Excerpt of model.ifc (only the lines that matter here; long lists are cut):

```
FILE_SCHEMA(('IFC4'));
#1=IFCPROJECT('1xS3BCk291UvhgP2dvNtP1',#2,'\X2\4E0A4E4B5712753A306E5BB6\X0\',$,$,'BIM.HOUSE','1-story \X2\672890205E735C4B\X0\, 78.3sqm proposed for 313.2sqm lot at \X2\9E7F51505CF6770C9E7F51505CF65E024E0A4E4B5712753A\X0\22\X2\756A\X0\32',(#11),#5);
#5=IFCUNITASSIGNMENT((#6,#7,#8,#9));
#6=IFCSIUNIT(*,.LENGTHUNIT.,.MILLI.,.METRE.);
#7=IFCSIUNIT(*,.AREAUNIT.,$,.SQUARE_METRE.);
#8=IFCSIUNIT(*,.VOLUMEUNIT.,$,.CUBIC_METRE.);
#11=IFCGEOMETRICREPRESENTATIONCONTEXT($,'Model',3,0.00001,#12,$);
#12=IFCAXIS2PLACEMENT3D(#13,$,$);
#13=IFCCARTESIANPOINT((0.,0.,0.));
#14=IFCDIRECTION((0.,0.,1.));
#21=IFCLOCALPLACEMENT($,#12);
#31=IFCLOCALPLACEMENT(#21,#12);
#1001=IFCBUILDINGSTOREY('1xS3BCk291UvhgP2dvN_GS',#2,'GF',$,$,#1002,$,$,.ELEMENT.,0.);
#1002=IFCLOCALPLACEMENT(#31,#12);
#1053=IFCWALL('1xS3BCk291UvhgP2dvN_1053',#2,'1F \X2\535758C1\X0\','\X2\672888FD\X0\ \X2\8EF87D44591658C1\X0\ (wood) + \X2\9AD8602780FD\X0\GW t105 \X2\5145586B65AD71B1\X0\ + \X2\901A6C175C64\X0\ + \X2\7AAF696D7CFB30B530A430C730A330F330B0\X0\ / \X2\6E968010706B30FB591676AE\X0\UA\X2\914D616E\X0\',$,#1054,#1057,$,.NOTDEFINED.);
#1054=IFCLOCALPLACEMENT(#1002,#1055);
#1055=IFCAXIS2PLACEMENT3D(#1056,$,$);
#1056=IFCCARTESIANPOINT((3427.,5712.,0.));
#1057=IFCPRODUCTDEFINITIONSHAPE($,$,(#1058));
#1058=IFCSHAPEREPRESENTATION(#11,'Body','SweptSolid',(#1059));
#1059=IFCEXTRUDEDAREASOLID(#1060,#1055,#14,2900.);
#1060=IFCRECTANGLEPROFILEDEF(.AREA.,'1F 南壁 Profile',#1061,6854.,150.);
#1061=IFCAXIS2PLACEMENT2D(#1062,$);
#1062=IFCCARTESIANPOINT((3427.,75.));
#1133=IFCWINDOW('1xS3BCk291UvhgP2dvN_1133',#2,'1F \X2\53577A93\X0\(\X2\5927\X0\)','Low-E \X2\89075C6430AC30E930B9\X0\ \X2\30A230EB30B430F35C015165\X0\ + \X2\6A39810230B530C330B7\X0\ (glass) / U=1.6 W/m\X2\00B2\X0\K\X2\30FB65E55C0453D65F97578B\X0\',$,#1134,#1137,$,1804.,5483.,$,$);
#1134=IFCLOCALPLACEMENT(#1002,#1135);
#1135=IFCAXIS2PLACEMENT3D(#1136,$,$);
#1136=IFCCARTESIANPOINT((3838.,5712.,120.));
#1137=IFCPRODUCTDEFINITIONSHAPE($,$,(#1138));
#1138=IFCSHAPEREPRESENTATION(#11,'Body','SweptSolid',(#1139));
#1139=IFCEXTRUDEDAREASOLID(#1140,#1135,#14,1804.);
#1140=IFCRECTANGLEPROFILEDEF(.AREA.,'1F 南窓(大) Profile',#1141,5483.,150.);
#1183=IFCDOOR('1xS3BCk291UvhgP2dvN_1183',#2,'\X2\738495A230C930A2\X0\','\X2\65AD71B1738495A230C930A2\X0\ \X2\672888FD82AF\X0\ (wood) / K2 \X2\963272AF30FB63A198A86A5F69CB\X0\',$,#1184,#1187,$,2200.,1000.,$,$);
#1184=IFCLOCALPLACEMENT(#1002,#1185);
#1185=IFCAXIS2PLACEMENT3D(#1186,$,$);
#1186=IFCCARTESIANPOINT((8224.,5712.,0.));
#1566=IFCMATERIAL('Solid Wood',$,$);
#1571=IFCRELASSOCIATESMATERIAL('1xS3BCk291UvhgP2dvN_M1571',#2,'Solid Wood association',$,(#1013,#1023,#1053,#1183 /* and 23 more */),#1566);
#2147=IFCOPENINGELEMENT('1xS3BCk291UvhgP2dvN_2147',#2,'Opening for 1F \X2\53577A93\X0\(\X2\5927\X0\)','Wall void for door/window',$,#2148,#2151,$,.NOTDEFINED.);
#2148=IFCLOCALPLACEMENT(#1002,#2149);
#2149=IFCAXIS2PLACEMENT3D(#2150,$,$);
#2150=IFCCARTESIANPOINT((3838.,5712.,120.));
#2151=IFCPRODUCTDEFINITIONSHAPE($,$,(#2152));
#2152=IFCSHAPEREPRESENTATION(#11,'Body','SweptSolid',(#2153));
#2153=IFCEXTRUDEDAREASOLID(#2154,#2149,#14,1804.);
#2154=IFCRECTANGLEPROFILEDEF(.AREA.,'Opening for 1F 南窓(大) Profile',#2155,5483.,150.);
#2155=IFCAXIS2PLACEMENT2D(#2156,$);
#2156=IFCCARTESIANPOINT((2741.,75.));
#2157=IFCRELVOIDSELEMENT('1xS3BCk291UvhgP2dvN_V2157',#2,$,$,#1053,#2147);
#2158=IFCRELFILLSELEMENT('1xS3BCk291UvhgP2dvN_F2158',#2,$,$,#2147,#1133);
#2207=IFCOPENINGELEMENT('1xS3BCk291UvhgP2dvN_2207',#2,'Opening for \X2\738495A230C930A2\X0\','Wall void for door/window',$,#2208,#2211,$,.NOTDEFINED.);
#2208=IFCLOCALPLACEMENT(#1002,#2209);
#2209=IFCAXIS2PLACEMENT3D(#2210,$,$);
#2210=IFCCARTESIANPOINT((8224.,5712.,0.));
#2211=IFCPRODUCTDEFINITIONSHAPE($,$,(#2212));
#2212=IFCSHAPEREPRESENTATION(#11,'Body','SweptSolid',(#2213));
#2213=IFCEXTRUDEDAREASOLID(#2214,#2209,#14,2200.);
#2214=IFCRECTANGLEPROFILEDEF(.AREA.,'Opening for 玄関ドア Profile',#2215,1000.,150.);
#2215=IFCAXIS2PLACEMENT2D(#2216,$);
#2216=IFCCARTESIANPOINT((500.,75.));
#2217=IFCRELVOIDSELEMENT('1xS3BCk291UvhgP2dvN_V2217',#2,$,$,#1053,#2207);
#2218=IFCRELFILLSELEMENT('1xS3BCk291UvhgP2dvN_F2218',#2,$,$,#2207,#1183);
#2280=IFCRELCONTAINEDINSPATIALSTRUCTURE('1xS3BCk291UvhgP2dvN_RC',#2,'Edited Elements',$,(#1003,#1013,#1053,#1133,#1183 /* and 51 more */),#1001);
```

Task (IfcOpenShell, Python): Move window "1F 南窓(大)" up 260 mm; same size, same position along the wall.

```python
import numpy as np
import ifcopenshell
import ifcopenshell.api.geometry
import ifcopenshell.util.placement
import ifcopenshell.util.unit

model = ifcopenshell.open("model.ifc")
unit_scale = ifcopenshell.util.unit.calculate_unit_scale(model)

window = model.by_id(1133)
opening = window.FillsVoids[0].RelatingOpeningElement
dz = 0.26 / unit_scale

shift = np.array([0.0, 0.0, dz])
# The window is not placed relative to its opening, so move both.
for product in (opening, window):
    matrix = ifcopenshell.util.placement.get_local_placement(product.ObjectPlacement)
    matrix[:3, 3] += shift
    ifcopenshell.api.geometry.edit_object_placement(model, product=product, matrix=matrix, is_si=False)

print(f"moved by {dz * unit_scale:+.3f} m")

model.write("model_v2.ifc")
```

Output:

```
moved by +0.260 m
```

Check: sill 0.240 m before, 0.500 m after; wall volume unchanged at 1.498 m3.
